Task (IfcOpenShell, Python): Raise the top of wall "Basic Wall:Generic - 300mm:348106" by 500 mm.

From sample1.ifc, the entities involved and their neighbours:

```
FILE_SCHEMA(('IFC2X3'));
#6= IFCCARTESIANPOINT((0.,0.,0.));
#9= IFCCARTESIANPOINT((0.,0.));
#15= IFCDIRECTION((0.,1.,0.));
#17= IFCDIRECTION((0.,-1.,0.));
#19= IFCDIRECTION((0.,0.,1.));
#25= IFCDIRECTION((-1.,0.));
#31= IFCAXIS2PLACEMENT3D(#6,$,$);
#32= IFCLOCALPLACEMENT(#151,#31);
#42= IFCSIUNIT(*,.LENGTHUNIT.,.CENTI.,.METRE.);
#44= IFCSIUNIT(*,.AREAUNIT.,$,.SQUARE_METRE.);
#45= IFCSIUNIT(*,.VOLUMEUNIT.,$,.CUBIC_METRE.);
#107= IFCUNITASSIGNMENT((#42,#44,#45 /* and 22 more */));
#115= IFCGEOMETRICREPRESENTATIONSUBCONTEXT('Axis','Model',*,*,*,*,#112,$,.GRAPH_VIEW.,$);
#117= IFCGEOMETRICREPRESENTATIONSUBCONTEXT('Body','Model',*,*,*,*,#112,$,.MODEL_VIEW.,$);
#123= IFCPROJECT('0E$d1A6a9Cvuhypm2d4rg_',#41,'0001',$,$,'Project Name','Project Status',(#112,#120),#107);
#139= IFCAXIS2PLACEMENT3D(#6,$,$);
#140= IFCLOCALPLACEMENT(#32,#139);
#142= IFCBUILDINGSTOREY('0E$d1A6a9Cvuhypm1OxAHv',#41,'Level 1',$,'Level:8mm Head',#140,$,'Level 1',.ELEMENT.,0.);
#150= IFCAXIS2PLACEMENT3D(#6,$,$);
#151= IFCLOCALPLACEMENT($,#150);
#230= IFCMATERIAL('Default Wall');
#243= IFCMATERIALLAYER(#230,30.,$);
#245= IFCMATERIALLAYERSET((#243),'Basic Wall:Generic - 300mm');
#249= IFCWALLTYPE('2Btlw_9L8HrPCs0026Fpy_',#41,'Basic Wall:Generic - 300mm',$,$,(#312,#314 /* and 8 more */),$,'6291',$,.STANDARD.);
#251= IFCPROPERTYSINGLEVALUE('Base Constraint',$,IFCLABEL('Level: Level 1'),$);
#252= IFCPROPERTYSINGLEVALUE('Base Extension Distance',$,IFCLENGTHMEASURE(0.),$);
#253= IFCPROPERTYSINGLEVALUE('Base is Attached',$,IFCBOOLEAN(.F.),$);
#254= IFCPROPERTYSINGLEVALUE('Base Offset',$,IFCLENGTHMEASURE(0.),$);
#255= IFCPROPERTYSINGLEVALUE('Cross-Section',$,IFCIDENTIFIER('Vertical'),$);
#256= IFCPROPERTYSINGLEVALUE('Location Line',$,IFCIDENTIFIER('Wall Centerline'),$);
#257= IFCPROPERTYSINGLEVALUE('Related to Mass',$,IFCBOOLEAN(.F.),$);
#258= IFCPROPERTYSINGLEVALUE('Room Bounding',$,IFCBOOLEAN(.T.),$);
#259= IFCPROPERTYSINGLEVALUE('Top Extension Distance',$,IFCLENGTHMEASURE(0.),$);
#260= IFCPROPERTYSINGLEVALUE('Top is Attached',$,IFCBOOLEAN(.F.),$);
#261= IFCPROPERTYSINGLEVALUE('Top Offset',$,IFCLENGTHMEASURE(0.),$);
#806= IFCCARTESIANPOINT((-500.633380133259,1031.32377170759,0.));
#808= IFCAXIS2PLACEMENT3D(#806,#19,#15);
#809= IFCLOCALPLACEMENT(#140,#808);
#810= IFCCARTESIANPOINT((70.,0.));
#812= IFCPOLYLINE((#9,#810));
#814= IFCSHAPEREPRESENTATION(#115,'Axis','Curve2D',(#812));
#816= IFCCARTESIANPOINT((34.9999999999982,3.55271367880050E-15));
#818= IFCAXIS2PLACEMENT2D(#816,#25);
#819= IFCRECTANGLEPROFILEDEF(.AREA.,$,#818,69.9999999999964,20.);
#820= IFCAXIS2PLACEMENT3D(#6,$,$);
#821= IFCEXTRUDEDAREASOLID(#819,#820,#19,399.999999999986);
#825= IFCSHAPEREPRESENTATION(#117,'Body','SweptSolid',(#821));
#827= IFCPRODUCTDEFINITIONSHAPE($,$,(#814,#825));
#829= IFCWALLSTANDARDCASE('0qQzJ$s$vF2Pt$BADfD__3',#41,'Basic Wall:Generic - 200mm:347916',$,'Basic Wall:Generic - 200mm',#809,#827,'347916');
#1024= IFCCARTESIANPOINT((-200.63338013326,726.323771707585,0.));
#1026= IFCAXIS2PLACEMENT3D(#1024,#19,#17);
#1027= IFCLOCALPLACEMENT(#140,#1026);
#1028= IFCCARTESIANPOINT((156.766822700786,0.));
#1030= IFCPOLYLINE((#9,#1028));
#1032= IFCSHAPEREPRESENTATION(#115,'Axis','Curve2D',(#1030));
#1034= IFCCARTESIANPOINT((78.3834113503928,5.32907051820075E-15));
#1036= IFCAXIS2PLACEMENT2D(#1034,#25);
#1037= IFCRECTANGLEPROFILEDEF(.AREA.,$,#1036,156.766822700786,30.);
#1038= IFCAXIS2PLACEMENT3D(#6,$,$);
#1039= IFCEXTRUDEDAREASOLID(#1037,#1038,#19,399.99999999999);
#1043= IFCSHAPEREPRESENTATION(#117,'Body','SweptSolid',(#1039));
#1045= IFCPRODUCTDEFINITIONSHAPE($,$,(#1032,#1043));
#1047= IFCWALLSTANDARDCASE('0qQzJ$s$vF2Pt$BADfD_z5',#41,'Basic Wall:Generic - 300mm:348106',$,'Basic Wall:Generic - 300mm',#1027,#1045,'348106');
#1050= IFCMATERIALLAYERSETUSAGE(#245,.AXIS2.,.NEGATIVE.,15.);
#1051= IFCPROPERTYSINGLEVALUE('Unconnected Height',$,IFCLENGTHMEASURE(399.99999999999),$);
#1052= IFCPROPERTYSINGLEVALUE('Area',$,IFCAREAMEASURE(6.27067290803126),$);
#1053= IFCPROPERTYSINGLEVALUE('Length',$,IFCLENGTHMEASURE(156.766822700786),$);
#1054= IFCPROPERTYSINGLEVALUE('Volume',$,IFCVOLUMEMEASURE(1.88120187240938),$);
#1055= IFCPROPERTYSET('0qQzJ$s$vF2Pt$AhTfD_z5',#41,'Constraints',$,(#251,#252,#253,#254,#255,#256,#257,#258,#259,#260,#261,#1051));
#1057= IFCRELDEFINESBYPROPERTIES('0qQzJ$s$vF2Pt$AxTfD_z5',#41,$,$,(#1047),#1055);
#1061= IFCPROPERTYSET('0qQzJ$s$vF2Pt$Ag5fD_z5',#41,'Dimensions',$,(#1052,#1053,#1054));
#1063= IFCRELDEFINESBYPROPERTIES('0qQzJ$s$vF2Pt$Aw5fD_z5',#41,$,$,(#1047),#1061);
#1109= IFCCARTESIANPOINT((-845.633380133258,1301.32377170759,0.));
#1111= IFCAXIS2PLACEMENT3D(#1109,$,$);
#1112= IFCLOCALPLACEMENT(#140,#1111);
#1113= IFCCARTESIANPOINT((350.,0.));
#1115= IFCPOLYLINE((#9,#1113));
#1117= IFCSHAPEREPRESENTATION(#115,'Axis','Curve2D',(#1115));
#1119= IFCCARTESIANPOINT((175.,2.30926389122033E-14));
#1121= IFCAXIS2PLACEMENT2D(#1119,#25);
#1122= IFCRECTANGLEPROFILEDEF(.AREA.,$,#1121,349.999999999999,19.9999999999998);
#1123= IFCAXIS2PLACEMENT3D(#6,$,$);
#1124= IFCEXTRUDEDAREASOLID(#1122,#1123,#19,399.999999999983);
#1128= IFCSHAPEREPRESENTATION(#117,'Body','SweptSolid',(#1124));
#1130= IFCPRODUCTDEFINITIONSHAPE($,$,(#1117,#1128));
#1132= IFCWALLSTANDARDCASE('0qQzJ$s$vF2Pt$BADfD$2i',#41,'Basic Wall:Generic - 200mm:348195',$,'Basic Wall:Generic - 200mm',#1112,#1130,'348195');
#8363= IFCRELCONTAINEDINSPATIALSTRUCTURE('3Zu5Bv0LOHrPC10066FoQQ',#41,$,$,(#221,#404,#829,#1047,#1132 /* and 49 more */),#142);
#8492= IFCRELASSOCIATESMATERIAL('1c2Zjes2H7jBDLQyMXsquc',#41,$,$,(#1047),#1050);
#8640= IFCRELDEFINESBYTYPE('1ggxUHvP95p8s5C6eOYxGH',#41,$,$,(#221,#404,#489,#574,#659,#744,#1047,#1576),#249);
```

```python
import ifcopenshell
import ifcopenshell.api.pset
import ifcopenshell.geom
import ifcopenshell.util.element
import ifcopenshell.util.representation
import ifcopenshell.util.shape
import ifcopenshell.util.unit

model = ifcopenshell.open("sample1.ifc")
unit_scale = ifcopenshell.util.unit.calculate_unit_scale(model)
area_scale = ifcopenshell.util.unit.calculate_unit_scale(model, "AREAUNIT")
volume_scale = ifcopenshell.util.unit.calculate_unit_scale(model, "VOLUMEUNIT")
settings = ifcopenshell.geom.settings()


def volume(element):
    """Net volume in cubic metres, openings subtracted."""
    shape = ifcopenshell.geom.create_shape(settings, element)
    return ifcopenshell.util.shape.get_volume(shape.geometry)


wall = model.by_guid("0qQzJ$s$vF2Pt$BADfD_z5")
before = volume(wall)

body = ifcopenshell.util.representation.get_representation(wall, "Model", "Body")
solid = body.Items[0]
old_height = solid.Depth
solid.Depth += 0.5 / unit_scale
after = volume(wall)
thickness = 0.3  # wall thickness in metres

# Update the stored height, areas and volumes.
pset = model.by_id(ifcopenshell.util.element.get_pset(wall, "Constraints", should_inherit=False)["id"])
ifcopenshell.api.pset.edit_pset(model, pset=pset, properties={
    "Unconnected Height": model.create_entity("IfcLengthMeasure", solid.Depth),
})
pset = model.by_id(ifcopenshell.util.element.get_pset(wall, "Dimensions", should_inherit=False)["id"])
ifcopenshell.api.pset.edit_pset(model, pset=pset, properties={
    "Area": model.create_entity("IfcAreaMeasure", after / thickness / area_scale),
    "Volume": model.create_entity("IfcVolumeMeasure", after / volume_scale),
})

print(f"height {old_height:g} -> {solid.Depth:g}, volume {before:.3f} -> {after:.3f} m3")

model.write("sample1-out.ifc")
```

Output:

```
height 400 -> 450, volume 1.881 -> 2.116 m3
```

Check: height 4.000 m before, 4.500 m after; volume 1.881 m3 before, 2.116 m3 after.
